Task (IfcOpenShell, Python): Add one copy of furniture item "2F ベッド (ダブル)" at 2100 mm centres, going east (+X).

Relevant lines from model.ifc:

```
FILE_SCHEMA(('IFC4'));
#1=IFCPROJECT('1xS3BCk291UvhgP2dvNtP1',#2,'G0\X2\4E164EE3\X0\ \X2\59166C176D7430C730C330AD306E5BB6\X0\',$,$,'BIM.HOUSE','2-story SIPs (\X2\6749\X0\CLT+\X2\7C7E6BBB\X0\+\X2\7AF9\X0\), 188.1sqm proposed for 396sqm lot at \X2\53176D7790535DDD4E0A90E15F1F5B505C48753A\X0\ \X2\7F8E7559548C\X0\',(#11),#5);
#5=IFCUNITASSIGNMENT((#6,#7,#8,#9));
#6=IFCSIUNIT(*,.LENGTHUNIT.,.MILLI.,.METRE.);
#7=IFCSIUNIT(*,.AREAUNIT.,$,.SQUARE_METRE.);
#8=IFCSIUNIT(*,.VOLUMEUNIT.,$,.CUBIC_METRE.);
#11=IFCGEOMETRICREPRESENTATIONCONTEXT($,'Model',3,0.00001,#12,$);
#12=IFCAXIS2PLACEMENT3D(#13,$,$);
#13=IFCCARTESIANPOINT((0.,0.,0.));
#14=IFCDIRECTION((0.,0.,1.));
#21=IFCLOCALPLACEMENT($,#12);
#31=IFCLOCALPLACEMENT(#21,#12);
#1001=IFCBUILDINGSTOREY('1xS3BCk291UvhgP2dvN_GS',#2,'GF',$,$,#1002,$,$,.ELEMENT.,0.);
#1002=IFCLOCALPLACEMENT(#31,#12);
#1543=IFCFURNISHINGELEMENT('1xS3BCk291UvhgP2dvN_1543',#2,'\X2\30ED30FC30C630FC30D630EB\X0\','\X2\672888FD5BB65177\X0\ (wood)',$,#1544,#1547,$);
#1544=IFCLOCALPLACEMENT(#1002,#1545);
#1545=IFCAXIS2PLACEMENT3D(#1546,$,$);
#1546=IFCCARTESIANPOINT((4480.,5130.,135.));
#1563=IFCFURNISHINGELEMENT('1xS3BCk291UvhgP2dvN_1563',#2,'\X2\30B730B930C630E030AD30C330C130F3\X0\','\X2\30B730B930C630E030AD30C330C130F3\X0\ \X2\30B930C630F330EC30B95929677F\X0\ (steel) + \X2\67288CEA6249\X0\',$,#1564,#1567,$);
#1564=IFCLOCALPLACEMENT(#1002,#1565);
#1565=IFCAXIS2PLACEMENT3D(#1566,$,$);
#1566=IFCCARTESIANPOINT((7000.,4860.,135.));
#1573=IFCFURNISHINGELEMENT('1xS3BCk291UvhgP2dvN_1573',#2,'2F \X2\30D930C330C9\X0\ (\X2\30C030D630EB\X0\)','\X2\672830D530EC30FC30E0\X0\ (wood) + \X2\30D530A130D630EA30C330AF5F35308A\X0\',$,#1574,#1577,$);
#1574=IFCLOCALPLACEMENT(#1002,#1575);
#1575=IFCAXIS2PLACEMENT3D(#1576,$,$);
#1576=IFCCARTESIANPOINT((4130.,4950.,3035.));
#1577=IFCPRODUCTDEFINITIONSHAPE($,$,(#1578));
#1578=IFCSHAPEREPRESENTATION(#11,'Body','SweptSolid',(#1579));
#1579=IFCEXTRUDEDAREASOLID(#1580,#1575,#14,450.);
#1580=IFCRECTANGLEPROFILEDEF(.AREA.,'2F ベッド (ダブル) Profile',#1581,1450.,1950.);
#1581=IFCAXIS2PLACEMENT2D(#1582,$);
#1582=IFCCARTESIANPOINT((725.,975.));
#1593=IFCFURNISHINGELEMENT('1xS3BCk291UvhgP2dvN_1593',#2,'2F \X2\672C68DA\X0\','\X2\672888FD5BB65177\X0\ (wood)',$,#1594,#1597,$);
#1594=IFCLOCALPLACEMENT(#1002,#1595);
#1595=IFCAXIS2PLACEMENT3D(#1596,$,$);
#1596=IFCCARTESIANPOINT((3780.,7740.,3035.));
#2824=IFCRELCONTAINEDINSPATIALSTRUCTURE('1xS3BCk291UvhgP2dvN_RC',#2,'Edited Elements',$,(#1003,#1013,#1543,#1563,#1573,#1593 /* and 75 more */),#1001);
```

```python
import numpy as np
import ifcopenshell
import ifcopenshell.api.geometry
import ifcopenshell.api.root
import ifcopenshell.util.element
import ifcopenshell.util.placement

model = ifcopenshell.open("model.ifc")


def reuse_history(source, copy):
    """copy_class also copies each property set's owner history, people and application; keep the originals."""
    for rel in copy.IsDefinedBy:
        if rel.is_a("IfcRelDefinesByProperties") and (history := rel.RelatingPropertyDefinition.OwnerHistory):
            rel.RelatingPropertyDefinition.OwnerHistory = source.OwnerHistory
            ifcopenshell.util.element.remove_deep2(model, history)


source = model.by_id(1573)
base = ifcopenshell.util.placement.get_local_placement(source.ObjectPlacement)
step = np.array([1.0, 0.0, 0.0]) * 2100.0

for i in range(1, 2):
    copy = ifcopenshell.api.root.copy_class(model, product=source)
    copy.Representation = ifcopenshell.util.element.copy_deep(
        model, source.Representation, exclude=["IfcGeometricRepresentationContext", "IfcRepresentationMap"]
    )
    reuse_history(source, copy)
    matrix = base.copy()
    matrix[:3, 3] += i * step
    print("added at", matrix[:3, 3].round(3) + 0.0)
    ifcopenshell.api.geometry.edit_object_placement(model, product=copy, matrix=matrix, is_si=False)

model.write("model_updated.ifc")
```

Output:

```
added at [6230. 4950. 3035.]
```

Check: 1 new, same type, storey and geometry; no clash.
